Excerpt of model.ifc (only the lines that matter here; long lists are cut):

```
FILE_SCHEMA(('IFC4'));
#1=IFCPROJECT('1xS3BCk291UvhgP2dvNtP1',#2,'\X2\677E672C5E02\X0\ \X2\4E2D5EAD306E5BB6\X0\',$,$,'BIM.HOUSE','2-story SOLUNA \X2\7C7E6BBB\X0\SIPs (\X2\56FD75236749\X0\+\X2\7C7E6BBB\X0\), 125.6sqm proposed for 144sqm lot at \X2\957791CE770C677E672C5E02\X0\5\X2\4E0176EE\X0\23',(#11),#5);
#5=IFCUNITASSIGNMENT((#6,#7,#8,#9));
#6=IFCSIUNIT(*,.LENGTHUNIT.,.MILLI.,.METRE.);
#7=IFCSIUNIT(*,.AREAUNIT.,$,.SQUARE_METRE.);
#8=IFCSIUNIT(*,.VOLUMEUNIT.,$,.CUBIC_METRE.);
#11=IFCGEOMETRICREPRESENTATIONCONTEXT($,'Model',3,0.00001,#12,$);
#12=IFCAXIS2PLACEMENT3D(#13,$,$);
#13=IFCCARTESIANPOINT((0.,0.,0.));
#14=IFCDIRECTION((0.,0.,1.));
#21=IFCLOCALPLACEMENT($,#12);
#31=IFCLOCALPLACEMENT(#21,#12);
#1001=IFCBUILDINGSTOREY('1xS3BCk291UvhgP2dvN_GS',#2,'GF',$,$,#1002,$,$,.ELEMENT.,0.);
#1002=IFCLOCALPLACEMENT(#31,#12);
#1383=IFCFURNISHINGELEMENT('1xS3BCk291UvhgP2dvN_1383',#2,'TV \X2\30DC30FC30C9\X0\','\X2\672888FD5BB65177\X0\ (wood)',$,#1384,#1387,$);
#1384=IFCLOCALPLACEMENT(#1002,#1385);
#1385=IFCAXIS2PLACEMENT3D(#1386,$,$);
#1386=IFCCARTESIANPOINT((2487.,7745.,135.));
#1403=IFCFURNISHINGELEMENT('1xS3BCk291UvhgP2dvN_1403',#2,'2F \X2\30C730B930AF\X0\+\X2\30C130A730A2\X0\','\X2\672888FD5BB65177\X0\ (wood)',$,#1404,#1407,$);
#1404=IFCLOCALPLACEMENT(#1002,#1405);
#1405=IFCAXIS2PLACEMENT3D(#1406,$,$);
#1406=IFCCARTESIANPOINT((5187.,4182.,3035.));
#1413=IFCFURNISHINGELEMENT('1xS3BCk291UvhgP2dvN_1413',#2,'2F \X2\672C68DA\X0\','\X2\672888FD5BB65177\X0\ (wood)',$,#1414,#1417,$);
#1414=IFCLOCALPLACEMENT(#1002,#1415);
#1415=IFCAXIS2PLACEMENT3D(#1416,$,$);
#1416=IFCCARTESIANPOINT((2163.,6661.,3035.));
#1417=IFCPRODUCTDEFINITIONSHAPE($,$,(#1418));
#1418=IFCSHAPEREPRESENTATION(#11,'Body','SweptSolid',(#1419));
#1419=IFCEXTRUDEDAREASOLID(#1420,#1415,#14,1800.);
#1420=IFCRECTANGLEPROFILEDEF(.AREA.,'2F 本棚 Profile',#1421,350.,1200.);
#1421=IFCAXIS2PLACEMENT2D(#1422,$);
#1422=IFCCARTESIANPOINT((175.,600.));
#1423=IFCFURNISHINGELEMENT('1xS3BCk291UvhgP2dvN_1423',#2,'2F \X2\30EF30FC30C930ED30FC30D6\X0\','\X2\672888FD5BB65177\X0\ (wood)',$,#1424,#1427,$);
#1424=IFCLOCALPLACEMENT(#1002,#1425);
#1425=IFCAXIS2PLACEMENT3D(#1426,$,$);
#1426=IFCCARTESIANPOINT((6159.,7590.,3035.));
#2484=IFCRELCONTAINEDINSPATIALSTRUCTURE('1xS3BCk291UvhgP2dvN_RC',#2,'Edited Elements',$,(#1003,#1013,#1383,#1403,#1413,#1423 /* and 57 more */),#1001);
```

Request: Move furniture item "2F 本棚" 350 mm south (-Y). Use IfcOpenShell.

```python
import ifcopenshell
import ifcopenshell.api.geometry
import ifcopenshell.util.placement
import ifcopenshell.util.unit

model = ifcopenshell.open("model.ifc")
unit_scale = ifcopenshell.util.unit.calculate_unit_scale(model)

item = model.by_guid("1xS3BCk291UvhgP2dvN_1413")
matrix = ifcopenshell.util.placement.get_local_placement(item.ObjectPlacement)
matrix[1, 3] -= 0.35 / unit_scale
ifcopenshell.api.geometry.edit_object_placement(model, product=item, matrix=matrix, is_si=False)

print(ifcopenshell.util.placement.get_local_placement(item.ObjectPlacement).round(3) + 0.0)

model.write("model_edited.ifc")
```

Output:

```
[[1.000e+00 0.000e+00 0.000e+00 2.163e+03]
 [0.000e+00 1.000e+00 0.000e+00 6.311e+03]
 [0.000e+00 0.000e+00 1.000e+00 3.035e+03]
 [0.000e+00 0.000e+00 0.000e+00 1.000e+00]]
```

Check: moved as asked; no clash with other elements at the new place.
